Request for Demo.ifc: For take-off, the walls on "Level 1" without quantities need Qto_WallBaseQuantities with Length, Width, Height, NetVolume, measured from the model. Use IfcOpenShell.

First a look at what the model holds.

```python
import ifcopenshell
import ifcopenshell.util.element
import ifcopenshell.util.unit

model = ifcopenshell.open("Demo.ifc")
print(model.schema)
for unit_type in ("LENGTHUNIT", "AREAUNIT", "VOLUMEUNIT"):
    print(unit_type, ifcopenshell.util.unit.calculate_unit_scale(model, unit_type))
storey = next(s for s in model.by_type("IfcBuildingStorey") if s.Name == "Level 1")
walls = [e for e in ifcopenshell.util.element.get_decomposition(storey) if e.is_a("IfcWall")]
for e in sorted(walls, key=lambda e: e.id()):
    print(e.id(), e.is_a(), e.Name, list(ifcopenshell.util.element.get_psets(e, qtos_only=True)), sep=" | ")
```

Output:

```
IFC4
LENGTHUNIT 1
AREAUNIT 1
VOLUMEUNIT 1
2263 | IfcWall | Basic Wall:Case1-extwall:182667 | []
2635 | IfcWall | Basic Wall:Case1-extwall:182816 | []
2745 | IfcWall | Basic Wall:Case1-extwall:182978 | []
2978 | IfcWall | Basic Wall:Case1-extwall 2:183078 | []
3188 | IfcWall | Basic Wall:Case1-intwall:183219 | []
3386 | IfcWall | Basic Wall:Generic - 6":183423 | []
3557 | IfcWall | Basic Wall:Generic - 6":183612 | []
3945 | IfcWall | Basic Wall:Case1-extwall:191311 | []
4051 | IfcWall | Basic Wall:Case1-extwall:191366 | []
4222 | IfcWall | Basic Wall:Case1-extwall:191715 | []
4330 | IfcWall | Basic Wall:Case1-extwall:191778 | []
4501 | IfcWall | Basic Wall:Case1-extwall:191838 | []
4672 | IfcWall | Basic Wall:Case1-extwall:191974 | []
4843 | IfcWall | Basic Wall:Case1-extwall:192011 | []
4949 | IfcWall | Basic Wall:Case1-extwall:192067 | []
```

```python
import ifcopenshell
import ifcopenshell.api.pset
import ifcopenshell.geom
import ifcopenshell.util.element
import ifcopenshell.util.shape
import ifcopenshell.util.unit

model = ifcopenshell.open("Demo.ifc")
unit_scale = ifcopenshell.util.unit.calculate_unit_scale(model)
volume_scale = ifcopenshell.util.unit.calculate_unit_scale(model, "VOLUMEUNIT")
settings = ifcopenshell.geom.settings()

storey = next(s for s in model.by_type("IfcBuildingStorey") if s.Name == "Level 1")
walls = [e for e in ifcopenshell.util.element.get_decomposition(storey) if e.is_a("IfcWall")]

for e in sorted(walls, key=lambda e: e.id()):
    if ifcopenshell.util.element.get_psets(e, qtos_only=True, should_inherit=False):
        continue
    # Geometry comes back in metres, in the element's own axes.
    shape = ifcopenshell.geom.create_shape(settings, e)
    values = {
        "Length": ifcopenshell.util.shape.get_x(shape.geometry) / unit_scale,
        "Width": ifcopenshell.util.shape.get_y(shape.geometry) / unit_scale,
        "Height": ifcopenshell.util.shape.get_z(shape.geometry) / unit_scale,
        "NetVolume": ifcopenshell.util.shape.get_volume(shape.geometry) / volume_scale,
    }
    qto = ifcopenshell.api.pset.add_qto(model, product=e, name="Qto_WallBaseQuantities")
    ifcopenshell.api.pset.edit_qto(model, qto=qto, properties=values)
    print(e.id(), {k: round(v, 3) for k, v in values.items()})

model.write("Demo_rev.ifc")
```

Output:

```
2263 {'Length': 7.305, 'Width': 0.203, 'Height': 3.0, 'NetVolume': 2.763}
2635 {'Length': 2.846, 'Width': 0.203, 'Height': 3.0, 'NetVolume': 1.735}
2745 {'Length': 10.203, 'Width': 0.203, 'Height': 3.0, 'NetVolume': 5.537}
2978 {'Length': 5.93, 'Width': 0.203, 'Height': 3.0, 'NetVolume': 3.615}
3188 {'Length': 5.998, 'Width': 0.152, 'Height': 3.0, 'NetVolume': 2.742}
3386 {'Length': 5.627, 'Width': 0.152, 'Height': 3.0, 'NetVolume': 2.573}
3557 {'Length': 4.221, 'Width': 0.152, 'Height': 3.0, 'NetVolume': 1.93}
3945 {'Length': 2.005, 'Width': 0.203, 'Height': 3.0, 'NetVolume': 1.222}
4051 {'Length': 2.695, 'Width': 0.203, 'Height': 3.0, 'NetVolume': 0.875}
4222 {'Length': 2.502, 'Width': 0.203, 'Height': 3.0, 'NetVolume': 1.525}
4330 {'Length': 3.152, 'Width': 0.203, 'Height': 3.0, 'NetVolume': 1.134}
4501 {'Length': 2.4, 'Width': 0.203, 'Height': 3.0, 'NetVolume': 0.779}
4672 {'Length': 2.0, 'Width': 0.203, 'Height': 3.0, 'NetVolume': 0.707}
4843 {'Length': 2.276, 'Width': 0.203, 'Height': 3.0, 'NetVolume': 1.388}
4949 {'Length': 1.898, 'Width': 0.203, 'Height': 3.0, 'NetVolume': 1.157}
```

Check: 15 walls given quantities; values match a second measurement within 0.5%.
